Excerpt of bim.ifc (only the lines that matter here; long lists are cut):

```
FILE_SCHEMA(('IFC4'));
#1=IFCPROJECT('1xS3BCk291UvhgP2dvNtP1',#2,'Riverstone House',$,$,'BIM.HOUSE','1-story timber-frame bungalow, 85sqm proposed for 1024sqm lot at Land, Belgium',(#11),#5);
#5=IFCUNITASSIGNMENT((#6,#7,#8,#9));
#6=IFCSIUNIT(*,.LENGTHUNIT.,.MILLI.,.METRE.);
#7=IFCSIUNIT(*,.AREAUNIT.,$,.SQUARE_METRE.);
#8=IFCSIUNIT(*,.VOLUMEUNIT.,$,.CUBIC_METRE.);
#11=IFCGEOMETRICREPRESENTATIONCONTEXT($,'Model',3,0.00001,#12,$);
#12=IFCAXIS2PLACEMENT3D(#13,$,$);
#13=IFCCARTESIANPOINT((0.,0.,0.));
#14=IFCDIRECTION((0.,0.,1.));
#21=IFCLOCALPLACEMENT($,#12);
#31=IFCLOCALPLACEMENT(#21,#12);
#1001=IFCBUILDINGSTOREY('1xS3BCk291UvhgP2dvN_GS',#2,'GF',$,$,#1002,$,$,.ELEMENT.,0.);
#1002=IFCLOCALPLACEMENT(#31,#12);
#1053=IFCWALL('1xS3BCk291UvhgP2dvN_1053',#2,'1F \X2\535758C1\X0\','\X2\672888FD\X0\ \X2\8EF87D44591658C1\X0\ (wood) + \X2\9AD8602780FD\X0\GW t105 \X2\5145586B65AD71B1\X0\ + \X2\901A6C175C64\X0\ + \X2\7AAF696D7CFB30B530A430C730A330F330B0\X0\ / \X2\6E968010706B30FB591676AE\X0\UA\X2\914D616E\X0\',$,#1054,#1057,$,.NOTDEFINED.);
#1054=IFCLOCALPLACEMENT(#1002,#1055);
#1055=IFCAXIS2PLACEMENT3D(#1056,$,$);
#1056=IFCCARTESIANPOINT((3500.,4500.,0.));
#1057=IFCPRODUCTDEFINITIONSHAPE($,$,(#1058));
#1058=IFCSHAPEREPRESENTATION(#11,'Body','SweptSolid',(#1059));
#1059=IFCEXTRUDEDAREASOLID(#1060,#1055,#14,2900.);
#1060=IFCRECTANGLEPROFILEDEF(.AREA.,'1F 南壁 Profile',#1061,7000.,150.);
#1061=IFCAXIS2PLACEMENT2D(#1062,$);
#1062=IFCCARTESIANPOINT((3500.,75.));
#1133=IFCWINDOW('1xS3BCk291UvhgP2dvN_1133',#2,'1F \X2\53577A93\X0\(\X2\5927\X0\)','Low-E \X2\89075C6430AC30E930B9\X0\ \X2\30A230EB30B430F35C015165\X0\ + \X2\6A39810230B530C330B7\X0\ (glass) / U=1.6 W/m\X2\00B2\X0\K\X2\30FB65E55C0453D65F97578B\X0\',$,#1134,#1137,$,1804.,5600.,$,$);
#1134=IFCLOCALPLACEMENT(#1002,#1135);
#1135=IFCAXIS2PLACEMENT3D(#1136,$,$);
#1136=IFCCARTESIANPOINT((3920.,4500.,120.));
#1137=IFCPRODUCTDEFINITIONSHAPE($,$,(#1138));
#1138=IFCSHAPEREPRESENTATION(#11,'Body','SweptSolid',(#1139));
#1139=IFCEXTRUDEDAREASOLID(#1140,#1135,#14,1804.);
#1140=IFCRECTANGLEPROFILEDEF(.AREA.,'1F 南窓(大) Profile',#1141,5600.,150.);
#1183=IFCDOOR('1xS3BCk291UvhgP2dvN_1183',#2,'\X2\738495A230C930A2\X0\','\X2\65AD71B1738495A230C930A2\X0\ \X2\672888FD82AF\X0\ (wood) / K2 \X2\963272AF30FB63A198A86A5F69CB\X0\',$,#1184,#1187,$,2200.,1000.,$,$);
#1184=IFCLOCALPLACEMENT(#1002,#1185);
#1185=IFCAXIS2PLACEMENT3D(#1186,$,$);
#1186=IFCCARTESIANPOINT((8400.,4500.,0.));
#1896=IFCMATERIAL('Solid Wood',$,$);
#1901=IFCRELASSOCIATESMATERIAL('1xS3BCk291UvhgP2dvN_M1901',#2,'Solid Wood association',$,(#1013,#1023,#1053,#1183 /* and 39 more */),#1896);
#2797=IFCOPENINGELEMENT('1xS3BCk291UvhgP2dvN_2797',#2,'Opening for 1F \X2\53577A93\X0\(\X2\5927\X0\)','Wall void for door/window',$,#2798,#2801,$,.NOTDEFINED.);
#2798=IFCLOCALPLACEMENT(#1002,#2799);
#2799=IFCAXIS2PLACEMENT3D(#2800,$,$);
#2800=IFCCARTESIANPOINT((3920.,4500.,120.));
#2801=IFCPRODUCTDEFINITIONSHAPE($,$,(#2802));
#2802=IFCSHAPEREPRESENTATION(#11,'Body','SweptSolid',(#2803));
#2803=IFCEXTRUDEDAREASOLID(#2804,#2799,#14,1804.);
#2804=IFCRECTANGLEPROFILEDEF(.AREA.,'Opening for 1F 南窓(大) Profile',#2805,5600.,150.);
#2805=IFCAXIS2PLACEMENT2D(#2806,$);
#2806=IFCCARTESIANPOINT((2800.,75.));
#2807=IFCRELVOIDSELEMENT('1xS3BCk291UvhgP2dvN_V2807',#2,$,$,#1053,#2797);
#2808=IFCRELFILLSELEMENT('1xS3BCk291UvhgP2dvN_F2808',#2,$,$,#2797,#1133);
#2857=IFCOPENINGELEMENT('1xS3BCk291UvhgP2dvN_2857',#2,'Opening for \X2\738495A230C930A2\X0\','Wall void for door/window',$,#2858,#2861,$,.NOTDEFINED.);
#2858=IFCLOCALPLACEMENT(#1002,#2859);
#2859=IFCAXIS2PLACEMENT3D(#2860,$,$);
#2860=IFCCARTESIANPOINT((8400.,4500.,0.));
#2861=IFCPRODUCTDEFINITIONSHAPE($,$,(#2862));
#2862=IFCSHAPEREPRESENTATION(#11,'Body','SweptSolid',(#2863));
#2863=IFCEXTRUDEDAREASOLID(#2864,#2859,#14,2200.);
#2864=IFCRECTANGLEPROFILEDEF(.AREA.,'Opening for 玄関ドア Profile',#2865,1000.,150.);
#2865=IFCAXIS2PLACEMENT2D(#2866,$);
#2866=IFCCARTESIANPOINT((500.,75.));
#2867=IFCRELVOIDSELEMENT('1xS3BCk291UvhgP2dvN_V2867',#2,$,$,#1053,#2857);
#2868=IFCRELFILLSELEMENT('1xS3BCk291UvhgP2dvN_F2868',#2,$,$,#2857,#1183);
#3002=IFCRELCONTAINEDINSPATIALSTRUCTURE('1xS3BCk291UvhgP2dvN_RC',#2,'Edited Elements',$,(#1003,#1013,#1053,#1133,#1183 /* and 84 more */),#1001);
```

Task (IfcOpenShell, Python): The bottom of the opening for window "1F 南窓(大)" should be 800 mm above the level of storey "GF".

```python
import numpy as np
import ifcopenshell
import ifcopenshell.api.geometry
import ifcopenshell.geom
import ifcopenshell.util.element
import ifcopenshell.util.placement
import ifcopenshell.util.shape
import ifcopenshell.util.unit

model = ifcopenshell.open("bim.ifc")
unit_scale = ifcopenshell.util.unit.calculate_unit_scale(model)

window = model.by_guid("1xS3BCk291UvhgP2dvN_1133")
opening = window.FillsVoids[0].RelatingOpeningElement
storey = ifcopenshell.util.element.get_container(window, ifc_class="IfcBuildingStorey")
level = ifcopenshell.util.placement.get_local_placement(storey.ObjectPlacement)[2, 3]

# The opening's origin need not be at the sill, so measure its lowest point.
shape = ifcopenshell.geom.create_shape(ifcopenshell.geom.settings(), opening)
bottom = ifcopenshell.util.shape.get_shape_bottom_elevation(shape, shape.geometry) / unit_scale
dz = level + 0.8 / unit_scale - bottom

shift = np.array([0.0, 0.0, dz])
# The window is not placed relative to its opening, so move both.
for product in (opening, window):
    matrix = ifcopenshell.util.placement.get_local_placement(product.ObjectPlacement)
    matrix[:3, 3] += shift
    ifcopenshell.api.geometry.edit_object_placement(model, product=product, matrix=matrix, is_si=False)

print(f"moved by {dz * unit_scale:+.3f} m")

model.write("bim_updated.ifc")
```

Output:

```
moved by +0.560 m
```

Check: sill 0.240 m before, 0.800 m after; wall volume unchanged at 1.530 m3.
